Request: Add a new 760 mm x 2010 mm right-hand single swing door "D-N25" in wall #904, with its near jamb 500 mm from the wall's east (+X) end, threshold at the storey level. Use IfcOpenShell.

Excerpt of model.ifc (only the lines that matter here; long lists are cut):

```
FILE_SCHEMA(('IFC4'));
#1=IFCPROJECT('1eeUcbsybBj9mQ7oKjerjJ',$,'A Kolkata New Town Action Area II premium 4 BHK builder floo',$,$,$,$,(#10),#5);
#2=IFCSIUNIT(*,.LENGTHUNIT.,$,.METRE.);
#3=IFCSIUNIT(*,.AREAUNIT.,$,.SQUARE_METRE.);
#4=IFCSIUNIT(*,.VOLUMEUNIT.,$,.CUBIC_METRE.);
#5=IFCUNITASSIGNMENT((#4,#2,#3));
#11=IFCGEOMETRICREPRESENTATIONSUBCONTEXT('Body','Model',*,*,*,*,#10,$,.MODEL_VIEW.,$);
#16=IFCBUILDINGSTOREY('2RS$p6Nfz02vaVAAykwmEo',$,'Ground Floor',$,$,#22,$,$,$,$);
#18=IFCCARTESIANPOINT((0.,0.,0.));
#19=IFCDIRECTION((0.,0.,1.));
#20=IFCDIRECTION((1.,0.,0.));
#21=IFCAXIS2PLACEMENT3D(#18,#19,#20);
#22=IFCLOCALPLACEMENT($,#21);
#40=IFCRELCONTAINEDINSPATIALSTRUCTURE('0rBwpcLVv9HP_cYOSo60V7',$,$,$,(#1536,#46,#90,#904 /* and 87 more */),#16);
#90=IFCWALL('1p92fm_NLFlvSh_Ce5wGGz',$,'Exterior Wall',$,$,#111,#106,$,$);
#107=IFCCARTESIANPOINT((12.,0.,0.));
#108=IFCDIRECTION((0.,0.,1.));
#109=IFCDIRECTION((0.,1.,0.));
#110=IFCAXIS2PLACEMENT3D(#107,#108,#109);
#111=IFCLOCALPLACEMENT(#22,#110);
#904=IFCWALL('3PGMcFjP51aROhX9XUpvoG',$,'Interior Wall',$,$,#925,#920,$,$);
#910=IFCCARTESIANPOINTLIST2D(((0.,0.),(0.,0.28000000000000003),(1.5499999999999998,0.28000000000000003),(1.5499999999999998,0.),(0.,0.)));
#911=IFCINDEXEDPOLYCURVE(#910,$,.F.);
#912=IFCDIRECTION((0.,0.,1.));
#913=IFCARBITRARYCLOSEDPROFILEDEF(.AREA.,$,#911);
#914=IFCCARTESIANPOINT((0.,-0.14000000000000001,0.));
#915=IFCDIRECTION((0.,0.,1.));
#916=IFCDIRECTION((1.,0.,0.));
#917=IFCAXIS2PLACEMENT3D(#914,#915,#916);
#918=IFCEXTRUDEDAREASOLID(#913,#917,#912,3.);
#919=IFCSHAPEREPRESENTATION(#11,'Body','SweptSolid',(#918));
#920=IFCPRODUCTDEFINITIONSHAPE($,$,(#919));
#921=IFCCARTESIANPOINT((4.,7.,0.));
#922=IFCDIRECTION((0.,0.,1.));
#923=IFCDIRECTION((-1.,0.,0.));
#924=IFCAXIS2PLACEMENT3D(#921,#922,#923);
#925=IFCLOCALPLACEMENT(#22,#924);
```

```python
import numpy as np
import ifcopenshell
import ifcopenshell.api.feature
import ifcopenshell.api.geometry
import ifcopenshell.api.root
import ifcopenshell.api.spatial
import ifcopenshell.geom
import ifcopenshell.util.element
import ifcopenshell.util.placement
import ifcopenshell.util.representation
import ifcopenshell.util.shape
import ifcopenshell.util.unit

model = ifcopenshell.open("model.ifc")
unit_scale = ifcopenshell.util.unit.calculate_unit_scale(model)
settings = ifcopenshell.geom.settings()


def volume(element):
    """Net volume in cubic metres, openings subtracted."""
    shape = ifcopenshell.geom.create_shape(settings, element)
    return ifcopenshell.util.shape.get_volume(shape.geometry)


wall = model.by_guid("3PGMcFjP51aROhX9XUpvoG")
storey = ifcopenshell.util.element.get_container(wall, ifc_class="IfcBuildingStorey")
context = ifcopenshell.util.representation.get_context(model, "Model", "Body", "MODEL_VIEW")
before = volume(wall)

width, height, from_end, sill = 0.76, 2.01, 0.5, 0.0  # metres

# The wall runs along its own X axis, and the end named is its -X end.
wall_shape = ifcopenshell.geom.create_shape(settings, wall)
x, y, z = ifcopenshell.util.shape.get_vertices(wall_shape.geometry).T
start = x.min() + from_end
face, thickness = float(y.min()), float(y.max() - y.min())
wall_matrix = ifcopenshell.util.placement.get_local_placement(wall.ObjectPlacement)
level = ifcopenshell.util.placement.get_local_placement(storey.ObjectPlacement)[2, 3]


def in_wall(x, y):
    """Placement at x, y metres in the wall's axes, at sill height."""
    matrix = wall_matrix.copy()
    matrix[:, 3] = wall_matrix @ np.array([x / unit_scale, y / unit_scale, 0.0, 1.0])
    matrix[2, 3] = level + sill / unit_scale
    return matrix


# Opening: a box that overshoots both wall faces by 50 mm.
opening = ifcopenshell.api.root.create_entity(model, ifc_class="IfcOpeningElement", predefined_type="OPENING")
box = ifcopenshell.api.geometry.add_wall_representation(
    model, context=context, length=width, height=height, thickness=thickness + 0.1
)
ifcopenshell.api.geometry.assign_representation(model, product=opening, representation=box)
ifcopenshell.api.geometry.edit_object_placement(model, product=opening, matrix=in_wall(start, face - 0.05), is_si=False)
ifcopenshell.api.feature.add_feature(model, feature=opening, element=wall)

door = ifcopenshell.api.root.create_entity(model, ifc_class="IfcDoor", name="D-N25", predefined_type="DOOR")
door.OverallWidth, door.OverallHeight = width / unit_scale, height / unit_scale
door.OperationType = "SINGLE_SWING_RIGHT"
body = ifcopenshell.api.geometry.add_door_representation(
    model,
    context=context,
    overall_width=door.OverallWidth,
    overall_height=door.OverallHeight,
    operation_type="SINGLE_SWING_RIGHT",
    lining_properties={"LiningDepth": thickness / unit_scale, "ThresholdDepth": thickness / unit_scale},
)
ifcopenshell.api.geometry.assign_representation(model, product=door, representation=body)
ifcopenshell.api.spatial.assign_container(model, products=[door], relating_structure=storey)
ifcopenshell.api.feature.add_filling(model, opening=opening, element=door)

# The lining spans the wall, so the door starts at the wall face.
ifcopenshell.api.geometry.edit_object_placement(model, product=door, matrix=in_wall(start, face), is_si=False)

after = volume(wall)

print(f"wall volume {before:.3f} -> {after:.3f} m3")

model.write("model_updated.ifc")
```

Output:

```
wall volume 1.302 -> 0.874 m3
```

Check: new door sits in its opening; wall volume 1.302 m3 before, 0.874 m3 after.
